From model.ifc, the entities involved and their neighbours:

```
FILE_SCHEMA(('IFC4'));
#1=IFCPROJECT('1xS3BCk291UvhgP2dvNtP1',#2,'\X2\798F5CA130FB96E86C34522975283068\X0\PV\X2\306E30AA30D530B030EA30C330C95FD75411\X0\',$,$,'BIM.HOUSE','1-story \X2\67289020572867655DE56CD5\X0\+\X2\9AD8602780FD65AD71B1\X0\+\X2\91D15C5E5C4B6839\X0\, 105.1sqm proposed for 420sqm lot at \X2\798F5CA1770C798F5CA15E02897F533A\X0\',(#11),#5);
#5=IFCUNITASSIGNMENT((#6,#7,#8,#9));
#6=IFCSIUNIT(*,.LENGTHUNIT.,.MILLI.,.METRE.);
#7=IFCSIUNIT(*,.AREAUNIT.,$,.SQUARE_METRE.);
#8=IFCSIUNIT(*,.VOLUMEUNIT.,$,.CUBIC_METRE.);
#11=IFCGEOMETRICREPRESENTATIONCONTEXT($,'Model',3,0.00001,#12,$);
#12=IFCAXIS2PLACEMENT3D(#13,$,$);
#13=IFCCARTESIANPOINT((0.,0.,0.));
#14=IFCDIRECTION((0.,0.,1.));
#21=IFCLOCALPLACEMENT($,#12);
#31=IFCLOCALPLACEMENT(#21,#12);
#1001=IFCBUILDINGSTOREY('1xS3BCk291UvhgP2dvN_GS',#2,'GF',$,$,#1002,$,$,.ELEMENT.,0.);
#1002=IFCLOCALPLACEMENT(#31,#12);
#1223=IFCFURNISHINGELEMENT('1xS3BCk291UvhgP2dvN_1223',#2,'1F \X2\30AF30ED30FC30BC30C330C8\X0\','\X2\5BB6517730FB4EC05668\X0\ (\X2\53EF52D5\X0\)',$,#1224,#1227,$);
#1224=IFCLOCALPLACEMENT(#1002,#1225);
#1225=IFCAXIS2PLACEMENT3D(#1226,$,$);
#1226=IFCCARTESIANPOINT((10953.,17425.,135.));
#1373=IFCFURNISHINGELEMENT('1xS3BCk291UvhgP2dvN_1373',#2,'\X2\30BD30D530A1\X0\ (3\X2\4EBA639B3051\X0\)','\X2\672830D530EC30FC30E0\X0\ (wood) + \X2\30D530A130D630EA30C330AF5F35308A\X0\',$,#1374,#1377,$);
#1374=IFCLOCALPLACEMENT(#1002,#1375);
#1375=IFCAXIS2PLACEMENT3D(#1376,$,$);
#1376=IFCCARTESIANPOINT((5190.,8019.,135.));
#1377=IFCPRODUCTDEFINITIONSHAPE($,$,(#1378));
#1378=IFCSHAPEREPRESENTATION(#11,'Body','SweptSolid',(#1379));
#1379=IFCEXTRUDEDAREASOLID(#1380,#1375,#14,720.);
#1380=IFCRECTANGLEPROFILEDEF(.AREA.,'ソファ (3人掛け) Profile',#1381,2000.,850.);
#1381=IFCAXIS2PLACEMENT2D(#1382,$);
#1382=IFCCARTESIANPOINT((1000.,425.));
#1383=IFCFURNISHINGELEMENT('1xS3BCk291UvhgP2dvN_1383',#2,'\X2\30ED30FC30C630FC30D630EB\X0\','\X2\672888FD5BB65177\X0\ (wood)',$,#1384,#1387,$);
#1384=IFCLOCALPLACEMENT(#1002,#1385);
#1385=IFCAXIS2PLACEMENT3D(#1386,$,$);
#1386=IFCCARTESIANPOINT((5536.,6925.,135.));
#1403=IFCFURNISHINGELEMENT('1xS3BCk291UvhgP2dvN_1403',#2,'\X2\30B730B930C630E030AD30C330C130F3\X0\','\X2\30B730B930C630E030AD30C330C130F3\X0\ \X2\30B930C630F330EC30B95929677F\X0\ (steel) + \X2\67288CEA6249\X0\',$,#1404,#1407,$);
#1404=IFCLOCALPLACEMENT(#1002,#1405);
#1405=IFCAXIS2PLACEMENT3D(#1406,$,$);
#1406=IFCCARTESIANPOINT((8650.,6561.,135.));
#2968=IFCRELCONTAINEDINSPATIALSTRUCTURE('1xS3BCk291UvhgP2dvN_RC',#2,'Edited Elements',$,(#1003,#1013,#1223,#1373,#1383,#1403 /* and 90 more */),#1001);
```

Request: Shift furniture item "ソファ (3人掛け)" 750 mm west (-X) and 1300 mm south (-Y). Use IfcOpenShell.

```python
import ifcopenshell
import ifcopenshell.api.geometry
import ifcopenshell.util.placement
import ifcopenshell.util.unit

model = ifcopenshell.open("model.ifc")
unit_scale = ifcopenshell.util.unit.calculate_unit_scale(model)

item = model.by_guid("1xS3BCk291UvhgP2dvN_1373")
matrix = ifcopenshell.util.placement.get_local_placement(item.ObjectPlacement)
matrix[0, 3] -= 0.75 / unit_scale
matrix[1, 3] -= 1.3 / unit_scale
ifcopenshell.api.geometry.edit_object_placement(model, product=item, matrix=matrix, is_si=False)

print(ifcopenshell.util.placement.get_local_placement(item.ObjectPlacement).round(3) + 0.0)

model.write("model_edited.ifc")
```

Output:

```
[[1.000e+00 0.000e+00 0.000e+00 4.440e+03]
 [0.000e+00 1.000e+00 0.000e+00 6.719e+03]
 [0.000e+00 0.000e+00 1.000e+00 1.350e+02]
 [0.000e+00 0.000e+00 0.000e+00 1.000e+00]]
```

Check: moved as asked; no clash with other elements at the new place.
